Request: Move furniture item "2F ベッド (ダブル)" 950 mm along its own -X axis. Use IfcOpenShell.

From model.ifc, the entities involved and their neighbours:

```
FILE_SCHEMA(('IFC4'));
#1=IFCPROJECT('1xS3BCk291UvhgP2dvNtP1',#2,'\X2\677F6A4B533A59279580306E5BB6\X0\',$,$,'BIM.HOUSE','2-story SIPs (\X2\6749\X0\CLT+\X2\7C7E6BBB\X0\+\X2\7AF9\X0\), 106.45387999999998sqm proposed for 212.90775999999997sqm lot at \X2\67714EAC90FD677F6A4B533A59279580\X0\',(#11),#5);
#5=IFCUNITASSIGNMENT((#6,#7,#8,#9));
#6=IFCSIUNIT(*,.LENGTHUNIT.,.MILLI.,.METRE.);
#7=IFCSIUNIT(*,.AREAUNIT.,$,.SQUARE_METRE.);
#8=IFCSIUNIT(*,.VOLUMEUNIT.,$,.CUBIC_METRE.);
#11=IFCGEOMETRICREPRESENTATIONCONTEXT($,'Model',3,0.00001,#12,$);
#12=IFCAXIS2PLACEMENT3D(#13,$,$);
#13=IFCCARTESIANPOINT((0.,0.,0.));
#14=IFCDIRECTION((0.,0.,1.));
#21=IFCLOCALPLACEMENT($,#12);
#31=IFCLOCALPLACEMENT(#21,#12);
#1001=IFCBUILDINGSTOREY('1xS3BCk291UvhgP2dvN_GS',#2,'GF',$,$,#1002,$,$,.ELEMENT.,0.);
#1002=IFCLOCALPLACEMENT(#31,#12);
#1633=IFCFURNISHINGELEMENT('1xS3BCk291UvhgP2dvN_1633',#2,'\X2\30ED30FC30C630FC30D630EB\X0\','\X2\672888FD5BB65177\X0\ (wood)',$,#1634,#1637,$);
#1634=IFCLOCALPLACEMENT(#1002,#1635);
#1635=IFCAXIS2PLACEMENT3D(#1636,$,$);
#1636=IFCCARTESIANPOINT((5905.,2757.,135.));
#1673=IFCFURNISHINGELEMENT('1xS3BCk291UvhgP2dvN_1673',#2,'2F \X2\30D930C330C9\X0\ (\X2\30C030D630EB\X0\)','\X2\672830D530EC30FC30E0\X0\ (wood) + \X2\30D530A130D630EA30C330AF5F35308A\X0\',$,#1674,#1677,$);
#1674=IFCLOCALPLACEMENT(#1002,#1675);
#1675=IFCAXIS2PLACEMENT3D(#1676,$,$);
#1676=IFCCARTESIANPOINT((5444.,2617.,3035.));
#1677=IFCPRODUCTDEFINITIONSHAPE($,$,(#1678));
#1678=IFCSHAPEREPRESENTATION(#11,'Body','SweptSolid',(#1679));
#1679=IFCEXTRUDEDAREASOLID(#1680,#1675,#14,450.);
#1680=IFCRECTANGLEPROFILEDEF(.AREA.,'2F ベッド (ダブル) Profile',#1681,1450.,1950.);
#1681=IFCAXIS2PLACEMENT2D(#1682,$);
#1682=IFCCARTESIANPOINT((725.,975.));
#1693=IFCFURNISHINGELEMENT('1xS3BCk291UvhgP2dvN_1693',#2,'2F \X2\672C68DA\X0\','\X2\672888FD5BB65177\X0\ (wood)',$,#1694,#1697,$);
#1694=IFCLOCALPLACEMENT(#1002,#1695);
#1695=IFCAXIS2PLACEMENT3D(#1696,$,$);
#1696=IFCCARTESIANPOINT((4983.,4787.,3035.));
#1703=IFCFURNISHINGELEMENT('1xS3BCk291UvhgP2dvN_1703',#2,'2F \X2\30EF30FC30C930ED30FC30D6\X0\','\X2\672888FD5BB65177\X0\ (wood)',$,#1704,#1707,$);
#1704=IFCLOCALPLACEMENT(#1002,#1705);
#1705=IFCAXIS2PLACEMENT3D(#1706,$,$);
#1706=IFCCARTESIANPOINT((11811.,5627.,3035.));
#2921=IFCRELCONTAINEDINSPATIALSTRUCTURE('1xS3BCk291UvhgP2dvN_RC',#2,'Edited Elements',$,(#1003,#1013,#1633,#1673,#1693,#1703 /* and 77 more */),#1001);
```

```python
import ifcopenshell
import ifcopenshell.api.geometry
import ifcopenshell.util.placement
import ifcopenshell.util.unit

model = ifcopenshell.open("model.ifc")
unit_scale = ifcopenshell.util.unit.calculate_unit_scale(model)

item = model.by_guid("1xS3BCk291UvhgP2dvN_1673")
matrix = ifcopenshell.util.placement.get_local_placement(item.ObjectPlacement)
matrix[:3, 3] -= matrix[:3, 0] * 0.95 / unit_scale
ifcopenshell.api.geometry.edit_object_placement(model, product=item, matrix=matrix, is_si=False)

print(ifcopenshell.util.placement.get_local_placement(item.ObjectPlacement).round(3) + 0.0)

model.write("model_v2.ifc")
```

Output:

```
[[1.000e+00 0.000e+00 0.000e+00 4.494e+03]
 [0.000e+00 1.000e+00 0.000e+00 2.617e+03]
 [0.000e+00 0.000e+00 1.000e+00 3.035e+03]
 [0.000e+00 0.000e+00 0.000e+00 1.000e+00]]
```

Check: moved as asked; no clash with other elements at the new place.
